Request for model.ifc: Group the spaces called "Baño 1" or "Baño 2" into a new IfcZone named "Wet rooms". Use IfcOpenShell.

First a look at what the model holds.

```python
import ifcopenshell

model = ifcopenshell.open("model.ifc")
print(model.schema)
seen = {}
for space in model.by_type("IfcSpace"):
    seen[space.LongName] = seen.get(space.LongName, 0) + 1
for name, count in sorted(seen.items(), key=str):
    print(count, "x", name)
print("zones:", [z.Name for z in model.by_type("IfcZone")][:20])
```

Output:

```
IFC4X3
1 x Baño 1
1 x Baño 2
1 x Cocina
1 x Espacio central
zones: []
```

```python
import ifcopenshell
import ifcopenshell.api.group
import ifcopenshell.api.root

model = ifcopenshell.open("model.ifc")

names = {"Baño 1", "Baño 2"}
spaces = [s for s in model.by_type("IfcSpace") if s.LongName in names]

zone = ifcopenshell.api.root.create_entity(model, ifc_class="IfcZone", name="Wet rooms")
ifcopenshell.api.group.assign_group(model, products=spaces, group=zone)
print(len(spaces), "spaces in", zone.Name)

model.write("model_rev.ifc")
```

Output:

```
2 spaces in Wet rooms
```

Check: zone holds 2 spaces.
